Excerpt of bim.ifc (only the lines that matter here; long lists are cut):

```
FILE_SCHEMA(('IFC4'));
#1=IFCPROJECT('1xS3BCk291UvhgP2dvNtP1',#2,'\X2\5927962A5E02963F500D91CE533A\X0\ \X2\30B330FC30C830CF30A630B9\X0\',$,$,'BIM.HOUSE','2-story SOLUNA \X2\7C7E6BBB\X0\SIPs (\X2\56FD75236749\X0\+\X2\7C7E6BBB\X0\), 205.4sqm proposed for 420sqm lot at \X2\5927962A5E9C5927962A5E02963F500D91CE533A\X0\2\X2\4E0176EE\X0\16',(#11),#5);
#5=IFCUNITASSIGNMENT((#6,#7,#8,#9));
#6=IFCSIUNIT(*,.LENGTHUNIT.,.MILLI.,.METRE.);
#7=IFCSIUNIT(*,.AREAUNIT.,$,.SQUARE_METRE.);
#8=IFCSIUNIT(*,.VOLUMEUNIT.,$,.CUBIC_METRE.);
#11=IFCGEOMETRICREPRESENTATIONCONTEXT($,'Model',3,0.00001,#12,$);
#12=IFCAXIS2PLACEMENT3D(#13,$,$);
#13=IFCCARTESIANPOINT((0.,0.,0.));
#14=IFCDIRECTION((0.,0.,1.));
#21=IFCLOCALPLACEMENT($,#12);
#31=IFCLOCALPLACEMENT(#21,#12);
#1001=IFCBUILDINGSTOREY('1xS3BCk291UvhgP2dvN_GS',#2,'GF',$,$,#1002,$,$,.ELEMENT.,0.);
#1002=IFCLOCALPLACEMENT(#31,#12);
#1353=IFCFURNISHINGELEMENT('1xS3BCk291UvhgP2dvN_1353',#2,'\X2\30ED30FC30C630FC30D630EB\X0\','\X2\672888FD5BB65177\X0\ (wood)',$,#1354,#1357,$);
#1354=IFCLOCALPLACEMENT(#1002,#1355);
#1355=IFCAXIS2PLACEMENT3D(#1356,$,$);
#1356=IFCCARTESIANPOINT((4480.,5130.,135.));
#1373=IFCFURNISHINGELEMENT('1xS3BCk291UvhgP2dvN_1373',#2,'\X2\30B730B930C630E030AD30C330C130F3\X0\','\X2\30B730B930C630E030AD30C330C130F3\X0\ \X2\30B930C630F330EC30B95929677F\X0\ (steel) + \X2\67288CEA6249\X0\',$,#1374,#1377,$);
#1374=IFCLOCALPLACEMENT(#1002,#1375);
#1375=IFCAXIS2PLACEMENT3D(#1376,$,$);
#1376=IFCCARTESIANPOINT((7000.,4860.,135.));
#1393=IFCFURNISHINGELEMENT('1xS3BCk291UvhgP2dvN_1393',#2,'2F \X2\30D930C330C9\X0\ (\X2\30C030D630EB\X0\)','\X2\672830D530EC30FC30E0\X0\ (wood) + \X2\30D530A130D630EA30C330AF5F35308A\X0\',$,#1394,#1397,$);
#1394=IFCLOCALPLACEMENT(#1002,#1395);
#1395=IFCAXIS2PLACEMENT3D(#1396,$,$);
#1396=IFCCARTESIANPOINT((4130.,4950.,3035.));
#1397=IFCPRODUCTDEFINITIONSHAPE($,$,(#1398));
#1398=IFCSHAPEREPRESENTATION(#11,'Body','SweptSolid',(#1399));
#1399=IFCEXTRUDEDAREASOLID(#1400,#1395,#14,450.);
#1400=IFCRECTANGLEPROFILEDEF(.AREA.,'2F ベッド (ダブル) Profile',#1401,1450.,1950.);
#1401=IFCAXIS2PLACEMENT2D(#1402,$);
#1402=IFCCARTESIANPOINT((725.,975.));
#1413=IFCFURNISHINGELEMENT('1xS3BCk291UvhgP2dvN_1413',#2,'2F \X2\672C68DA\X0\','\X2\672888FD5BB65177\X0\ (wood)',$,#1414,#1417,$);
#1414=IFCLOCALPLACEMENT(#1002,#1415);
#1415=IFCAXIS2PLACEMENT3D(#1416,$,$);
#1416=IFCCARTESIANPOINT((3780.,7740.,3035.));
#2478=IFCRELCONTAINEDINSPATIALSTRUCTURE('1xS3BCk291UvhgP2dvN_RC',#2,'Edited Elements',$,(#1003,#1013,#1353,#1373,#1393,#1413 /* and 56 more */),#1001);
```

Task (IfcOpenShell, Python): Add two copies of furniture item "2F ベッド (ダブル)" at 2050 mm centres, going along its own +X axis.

```python
import ifcopenshell
import ifcopenshell.api.geometry
import ifcopenshell.api.root
import ifcopenshell.util.element
import ifcopenshell.util.placement

model = ifcopenshell.open("bim.ifc")


def reuse_history(source, copy):
    """copy_class also copies each property set's owner history, people and application; keep the originals."""
    for rel in copy.IsDefinedBy:
        if rel.is_a("IfcRelDefinesByProperties") and (history := rel.RelatingPropertyDefinition.OwnerHistory):
            rel.RelatingPropertyDefinition.OwnerHistory = source.OwnerHistory
            ifcopenshell.util.element.remove_deep2(model, history)


source = model.by_guid("1xS3BCk291UvhgP2dvN_1393")
base = ifcopenshell.util.placement.get_local_placement(source.ObjectPlacement)
step = base[:3, 0] * 2050.0

for i in range(1, 3):
    copy = ifcopenshell.api.root.copy_class(model, product=source)
    copy.Representation = ifcopenshell.util.element.copy_deep(
        model, source.Representation, exclude=["IfcGeometricRepresentationContext", "IfcRepresentationMap"]
    )
    reuse_history(source, copy)
    matrix = base.copy()
    matrix[:3, 3] += i * step
    print("added at", matrix[:3, 3].round(3) + 0.0)
    ifcopenshell.api.geometry.edit_object_placement(model, product=copy, matrix=matrix, is_si=False)

model.write("bim-out.ifc")
```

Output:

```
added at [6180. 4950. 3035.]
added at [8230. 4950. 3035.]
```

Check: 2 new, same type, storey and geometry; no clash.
